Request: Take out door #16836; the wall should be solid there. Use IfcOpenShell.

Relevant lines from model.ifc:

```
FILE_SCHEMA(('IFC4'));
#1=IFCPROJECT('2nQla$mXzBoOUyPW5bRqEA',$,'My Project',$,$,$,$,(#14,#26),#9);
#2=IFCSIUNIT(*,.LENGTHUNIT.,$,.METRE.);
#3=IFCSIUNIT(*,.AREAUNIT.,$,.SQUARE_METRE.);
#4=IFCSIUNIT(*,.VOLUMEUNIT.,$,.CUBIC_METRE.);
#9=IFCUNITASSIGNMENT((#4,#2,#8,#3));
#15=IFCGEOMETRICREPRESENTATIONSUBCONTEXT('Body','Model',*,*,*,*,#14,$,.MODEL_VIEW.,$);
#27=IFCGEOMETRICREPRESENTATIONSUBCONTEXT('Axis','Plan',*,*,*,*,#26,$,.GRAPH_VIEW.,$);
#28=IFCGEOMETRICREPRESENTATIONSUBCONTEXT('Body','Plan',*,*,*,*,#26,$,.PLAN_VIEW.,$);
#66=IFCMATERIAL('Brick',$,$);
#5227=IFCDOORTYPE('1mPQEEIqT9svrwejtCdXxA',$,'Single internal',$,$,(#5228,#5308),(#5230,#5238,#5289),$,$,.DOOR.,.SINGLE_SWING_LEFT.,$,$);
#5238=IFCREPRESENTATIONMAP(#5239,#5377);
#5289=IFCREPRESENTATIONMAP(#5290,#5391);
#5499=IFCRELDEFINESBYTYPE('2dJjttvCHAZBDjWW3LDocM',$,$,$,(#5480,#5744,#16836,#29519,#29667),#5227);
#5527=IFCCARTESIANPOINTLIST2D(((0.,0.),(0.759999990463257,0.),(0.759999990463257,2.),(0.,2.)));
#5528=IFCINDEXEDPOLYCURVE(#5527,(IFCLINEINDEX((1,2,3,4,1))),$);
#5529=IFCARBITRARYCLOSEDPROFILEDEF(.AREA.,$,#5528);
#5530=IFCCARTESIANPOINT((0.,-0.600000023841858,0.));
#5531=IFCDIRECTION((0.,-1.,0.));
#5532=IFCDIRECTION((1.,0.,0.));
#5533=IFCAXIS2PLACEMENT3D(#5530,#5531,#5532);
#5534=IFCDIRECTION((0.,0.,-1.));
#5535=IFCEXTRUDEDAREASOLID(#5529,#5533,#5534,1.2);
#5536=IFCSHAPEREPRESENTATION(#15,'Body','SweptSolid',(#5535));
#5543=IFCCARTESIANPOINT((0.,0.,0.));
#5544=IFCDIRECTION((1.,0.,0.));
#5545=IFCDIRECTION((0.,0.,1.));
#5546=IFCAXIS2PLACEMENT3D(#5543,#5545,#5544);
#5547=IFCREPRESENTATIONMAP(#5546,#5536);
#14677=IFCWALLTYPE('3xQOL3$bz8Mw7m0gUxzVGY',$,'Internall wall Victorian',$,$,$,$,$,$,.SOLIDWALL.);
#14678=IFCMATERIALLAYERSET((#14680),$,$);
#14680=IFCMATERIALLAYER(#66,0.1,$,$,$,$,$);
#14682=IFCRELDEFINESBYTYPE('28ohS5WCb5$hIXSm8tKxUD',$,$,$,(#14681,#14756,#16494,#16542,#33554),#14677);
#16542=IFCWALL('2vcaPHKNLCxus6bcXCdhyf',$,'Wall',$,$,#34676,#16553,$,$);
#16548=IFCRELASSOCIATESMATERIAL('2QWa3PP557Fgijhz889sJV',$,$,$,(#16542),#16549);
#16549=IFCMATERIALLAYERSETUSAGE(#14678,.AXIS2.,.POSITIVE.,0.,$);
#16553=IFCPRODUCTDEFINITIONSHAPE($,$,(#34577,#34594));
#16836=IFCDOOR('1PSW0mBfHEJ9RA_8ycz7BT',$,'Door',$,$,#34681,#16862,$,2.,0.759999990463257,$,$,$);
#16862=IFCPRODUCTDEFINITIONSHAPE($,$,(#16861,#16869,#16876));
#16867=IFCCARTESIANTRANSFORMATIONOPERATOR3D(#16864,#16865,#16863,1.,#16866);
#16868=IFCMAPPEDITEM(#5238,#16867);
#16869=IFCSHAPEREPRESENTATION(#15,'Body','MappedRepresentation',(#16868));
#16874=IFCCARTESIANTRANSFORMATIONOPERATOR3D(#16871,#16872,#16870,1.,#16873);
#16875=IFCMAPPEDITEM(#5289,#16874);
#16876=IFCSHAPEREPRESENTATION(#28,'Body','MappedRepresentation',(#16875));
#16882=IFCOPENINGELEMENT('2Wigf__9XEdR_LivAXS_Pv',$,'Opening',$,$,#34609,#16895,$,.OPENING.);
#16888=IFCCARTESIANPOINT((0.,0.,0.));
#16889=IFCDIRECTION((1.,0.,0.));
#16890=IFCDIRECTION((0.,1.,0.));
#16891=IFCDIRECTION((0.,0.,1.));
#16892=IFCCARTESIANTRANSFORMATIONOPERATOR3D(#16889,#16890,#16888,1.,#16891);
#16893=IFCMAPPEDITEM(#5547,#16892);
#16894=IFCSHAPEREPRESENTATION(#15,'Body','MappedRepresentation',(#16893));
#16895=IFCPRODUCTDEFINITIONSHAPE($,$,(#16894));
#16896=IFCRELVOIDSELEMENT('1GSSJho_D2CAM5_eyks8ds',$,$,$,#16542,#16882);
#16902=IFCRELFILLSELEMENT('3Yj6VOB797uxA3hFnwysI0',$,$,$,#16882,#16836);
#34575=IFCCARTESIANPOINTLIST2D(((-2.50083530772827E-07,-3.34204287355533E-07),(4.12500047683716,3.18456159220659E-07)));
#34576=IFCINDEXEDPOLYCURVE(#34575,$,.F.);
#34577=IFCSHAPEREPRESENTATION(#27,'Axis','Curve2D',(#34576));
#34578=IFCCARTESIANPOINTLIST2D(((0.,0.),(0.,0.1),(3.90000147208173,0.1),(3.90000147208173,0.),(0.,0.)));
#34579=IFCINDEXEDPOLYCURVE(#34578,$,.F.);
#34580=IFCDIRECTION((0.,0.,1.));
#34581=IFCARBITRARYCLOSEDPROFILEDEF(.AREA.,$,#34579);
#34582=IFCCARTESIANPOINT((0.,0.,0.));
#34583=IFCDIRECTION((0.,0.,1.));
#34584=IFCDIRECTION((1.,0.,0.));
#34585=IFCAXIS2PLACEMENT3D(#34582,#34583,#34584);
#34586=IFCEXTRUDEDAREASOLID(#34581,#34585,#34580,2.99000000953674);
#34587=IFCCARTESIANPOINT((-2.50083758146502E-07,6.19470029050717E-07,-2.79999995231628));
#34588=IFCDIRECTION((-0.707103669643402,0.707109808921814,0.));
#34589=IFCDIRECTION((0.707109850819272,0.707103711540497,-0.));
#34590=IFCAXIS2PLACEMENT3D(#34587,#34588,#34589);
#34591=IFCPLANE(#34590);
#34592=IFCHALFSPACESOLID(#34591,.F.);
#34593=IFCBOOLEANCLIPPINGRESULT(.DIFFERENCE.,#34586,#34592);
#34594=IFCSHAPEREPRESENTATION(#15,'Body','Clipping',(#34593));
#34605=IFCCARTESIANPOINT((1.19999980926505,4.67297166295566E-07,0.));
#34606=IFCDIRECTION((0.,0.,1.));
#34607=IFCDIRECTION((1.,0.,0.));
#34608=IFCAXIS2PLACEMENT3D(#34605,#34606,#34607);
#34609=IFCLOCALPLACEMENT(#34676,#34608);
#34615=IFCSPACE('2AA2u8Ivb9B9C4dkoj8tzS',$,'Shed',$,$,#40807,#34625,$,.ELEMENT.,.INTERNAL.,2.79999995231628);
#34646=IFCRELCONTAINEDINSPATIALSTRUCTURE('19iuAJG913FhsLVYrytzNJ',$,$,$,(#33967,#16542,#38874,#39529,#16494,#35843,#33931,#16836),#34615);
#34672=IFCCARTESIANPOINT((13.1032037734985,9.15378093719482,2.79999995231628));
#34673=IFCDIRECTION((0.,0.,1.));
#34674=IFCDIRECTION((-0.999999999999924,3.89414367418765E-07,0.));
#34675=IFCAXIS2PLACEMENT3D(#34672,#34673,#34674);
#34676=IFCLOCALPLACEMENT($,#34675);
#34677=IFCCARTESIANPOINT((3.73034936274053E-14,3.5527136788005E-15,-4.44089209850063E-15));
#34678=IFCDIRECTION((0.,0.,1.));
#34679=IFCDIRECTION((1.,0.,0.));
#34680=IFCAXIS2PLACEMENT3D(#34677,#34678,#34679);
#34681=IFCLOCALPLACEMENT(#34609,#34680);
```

```python
import ifcopenshell
import ifcopenshell.api.feature
import ifcopenshell.api.root
import ifcopenshell.geom
import ifcopenshell.util.shape

model = ifcopenshell.open("model.ifc")
settings = ifcopenshell.geom.settings()


def volume(element):
    """Net volume in cubic metres, openings subtracted."""
    shape = ifcopenshell.geom.create_shape(settings, element)
    return ifcopenshell.util.shape.get_volume(shape.geometry)


door = model.by_guid("1PSW0mBfHEJ9RA_8ycz7BT")
opening = door.FillsVoids[0].RelatingOpeningElement
wall = opening.VoidsElements[0].RelatingBuildingElement
before = volume(wall)

ifcopenshell.api.root.remove_product(model, product=door)
ifcopenshell.api.feature.remove_feature(model, feature=opening)

after = volume(wall)

print(f"wall volume {before:.3f} -> {after:.3f} m3")

model.write("model_updated.ifc")
```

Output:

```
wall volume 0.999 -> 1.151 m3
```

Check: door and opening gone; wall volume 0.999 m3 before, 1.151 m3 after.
